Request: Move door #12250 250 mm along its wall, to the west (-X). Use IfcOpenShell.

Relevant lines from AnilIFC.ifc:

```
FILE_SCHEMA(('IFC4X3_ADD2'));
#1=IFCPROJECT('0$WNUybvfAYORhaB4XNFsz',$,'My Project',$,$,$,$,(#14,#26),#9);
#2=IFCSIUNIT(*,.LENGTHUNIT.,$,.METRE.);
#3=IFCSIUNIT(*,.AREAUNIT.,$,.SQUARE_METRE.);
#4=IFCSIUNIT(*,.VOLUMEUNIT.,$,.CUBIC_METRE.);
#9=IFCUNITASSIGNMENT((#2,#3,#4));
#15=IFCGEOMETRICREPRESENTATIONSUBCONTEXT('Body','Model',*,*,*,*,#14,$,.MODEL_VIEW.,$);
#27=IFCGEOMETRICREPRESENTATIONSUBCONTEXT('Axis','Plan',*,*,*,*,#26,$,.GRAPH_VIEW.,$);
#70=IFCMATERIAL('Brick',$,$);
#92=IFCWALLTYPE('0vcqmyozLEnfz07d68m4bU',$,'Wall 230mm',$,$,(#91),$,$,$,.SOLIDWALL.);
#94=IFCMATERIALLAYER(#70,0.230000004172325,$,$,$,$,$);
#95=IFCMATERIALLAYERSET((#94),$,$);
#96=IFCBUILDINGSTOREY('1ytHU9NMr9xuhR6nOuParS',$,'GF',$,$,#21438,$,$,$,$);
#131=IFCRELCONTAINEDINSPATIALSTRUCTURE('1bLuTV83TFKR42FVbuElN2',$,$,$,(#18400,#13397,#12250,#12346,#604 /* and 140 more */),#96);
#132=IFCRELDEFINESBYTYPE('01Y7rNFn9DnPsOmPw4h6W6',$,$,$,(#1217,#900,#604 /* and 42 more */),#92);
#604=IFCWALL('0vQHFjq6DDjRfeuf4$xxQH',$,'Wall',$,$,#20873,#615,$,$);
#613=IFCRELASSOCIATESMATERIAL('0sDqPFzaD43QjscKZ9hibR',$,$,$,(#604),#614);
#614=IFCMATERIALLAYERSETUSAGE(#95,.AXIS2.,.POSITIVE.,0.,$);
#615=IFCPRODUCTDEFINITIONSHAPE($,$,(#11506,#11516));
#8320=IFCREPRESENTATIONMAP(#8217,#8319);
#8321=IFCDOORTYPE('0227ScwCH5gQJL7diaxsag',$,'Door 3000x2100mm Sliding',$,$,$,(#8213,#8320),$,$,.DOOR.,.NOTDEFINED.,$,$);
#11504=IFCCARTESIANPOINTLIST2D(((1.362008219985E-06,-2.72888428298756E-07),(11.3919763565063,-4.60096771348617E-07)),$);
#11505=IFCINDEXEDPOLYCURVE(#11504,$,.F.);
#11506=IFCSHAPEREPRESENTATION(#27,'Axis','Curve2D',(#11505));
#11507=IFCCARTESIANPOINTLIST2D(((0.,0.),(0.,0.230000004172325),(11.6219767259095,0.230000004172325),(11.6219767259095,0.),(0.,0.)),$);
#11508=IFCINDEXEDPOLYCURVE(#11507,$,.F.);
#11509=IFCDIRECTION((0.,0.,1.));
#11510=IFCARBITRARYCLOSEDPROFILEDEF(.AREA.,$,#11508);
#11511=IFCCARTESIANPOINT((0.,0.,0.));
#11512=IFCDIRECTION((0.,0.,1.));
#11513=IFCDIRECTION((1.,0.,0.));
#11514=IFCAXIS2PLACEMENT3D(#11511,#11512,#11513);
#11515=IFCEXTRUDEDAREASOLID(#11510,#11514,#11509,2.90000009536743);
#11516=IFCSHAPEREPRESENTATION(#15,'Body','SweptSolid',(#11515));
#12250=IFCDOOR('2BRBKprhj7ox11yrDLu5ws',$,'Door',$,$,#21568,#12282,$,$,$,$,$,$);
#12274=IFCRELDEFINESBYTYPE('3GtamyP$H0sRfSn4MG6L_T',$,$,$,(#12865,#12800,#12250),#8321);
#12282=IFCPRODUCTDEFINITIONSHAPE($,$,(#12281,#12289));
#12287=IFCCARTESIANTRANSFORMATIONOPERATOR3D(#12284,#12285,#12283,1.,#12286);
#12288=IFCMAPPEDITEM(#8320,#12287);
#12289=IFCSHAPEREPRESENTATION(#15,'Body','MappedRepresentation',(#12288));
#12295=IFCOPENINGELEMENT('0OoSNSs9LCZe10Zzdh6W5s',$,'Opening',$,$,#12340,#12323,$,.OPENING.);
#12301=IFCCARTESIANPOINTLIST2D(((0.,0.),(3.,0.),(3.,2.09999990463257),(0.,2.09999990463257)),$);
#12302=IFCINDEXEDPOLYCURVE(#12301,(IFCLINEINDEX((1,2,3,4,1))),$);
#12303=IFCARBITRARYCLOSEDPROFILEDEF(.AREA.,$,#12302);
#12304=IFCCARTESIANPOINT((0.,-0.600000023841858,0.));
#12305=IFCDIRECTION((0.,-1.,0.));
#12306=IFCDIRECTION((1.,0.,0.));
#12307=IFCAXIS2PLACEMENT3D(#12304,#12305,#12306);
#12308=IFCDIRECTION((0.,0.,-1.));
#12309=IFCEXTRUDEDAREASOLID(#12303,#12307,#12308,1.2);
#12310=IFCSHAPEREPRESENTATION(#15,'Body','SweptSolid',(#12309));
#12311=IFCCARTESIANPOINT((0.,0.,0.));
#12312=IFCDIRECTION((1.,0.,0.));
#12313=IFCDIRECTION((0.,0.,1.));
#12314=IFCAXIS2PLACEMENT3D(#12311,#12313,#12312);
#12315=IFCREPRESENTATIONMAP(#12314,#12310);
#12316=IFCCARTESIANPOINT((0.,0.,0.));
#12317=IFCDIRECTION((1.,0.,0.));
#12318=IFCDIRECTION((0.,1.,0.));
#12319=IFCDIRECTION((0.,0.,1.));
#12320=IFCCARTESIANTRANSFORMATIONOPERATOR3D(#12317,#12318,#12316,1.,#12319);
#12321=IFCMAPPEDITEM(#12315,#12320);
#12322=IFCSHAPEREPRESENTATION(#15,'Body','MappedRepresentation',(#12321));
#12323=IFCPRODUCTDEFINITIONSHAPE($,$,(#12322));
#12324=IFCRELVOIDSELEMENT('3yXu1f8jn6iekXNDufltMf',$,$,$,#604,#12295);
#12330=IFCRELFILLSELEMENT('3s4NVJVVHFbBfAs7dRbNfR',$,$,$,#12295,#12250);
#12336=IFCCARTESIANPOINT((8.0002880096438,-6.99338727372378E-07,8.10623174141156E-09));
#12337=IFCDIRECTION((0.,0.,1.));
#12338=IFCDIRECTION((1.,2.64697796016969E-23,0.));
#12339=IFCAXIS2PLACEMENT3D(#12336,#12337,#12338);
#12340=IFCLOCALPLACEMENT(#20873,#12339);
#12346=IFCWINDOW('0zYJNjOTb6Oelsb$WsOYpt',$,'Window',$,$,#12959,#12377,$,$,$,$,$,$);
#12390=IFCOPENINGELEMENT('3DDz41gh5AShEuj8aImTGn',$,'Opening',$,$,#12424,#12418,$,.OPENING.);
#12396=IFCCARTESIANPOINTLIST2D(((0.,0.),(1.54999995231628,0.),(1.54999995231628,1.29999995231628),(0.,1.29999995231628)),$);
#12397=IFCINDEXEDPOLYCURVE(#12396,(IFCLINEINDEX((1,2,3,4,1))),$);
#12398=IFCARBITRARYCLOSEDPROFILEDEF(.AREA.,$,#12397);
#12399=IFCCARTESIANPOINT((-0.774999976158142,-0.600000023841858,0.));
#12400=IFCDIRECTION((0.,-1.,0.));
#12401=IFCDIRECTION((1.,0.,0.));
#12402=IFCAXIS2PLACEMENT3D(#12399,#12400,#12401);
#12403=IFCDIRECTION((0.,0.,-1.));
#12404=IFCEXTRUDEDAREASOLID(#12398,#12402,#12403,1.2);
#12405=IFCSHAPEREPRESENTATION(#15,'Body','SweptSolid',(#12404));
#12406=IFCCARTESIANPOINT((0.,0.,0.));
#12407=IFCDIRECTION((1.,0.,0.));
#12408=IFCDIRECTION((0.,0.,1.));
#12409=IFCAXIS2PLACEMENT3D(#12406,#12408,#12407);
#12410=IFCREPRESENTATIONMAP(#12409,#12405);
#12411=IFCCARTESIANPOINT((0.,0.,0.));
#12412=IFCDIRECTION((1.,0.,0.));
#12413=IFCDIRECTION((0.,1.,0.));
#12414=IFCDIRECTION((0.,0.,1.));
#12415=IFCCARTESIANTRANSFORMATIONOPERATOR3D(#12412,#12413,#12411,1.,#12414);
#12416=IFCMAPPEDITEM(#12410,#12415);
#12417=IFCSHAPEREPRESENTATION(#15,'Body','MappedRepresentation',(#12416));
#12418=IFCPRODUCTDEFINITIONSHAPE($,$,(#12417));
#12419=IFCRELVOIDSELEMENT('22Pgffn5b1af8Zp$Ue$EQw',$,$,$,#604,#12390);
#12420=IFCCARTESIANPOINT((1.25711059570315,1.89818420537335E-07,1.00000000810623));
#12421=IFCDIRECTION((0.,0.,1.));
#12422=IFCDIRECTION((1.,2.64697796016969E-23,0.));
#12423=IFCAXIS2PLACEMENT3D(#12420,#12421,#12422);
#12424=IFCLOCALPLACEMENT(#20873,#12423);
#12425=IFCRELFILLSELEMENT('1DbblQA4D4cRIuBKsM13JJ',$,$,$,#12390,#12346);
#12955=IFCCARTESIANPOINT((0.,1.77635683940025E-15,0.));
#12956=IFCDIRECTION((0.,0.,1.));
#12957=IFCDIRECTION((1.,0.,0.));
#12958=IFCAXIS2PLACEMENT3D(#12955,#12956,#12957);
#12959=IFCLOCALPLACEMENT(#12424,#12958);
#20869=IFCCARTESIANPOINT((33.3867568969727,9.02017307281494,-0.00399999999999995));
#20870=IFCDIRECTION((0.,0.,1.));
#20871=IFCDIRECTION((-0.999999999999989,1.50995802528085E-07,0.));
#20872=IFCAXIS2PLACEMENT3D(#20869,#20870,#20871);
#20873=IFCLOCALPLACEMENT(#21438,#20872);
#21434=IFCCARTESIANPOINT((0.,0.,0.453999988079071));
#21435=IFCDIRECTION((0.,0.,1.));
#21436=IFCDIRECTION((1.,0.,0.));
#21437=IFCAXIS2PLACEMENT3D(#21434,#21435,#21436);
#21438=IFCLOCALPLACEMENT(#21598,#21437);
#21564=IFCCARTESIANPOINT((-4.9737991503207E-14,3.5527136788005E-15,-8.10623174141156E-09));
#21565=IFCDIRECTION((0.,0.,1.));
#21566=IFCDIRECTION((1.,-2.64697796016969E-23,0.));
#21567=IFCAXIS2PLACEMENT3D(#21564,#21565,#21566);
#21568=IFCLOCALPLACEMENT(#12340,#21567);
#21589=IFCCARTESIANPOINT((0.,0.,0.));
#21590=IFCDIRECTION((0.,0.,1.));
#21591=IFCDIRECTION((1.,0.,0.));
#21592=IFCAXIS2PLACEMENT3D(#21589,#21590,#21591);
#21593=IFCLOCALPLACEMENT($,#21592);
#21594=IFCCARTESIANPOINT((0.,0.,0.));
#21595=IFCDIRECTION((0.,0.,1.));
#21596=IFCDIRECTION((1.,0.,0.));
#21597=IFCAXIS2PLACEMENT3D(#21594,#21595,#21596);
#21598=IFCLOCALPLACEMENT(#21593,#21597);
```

```python
import ifcopenshell
import ifcopenshell.api.geometry
import ifcopenshell.util.placement
import ifcopenshell.util.unit

model = ifcopenshell.open("AnilIFC.ifc")
unit_scale = ifcopenshell.util.unit.calculate_unit_scale(model)

door = model.by_guid("2BRBKprhj7ox11yrDLu5ws")
opening = door.FillsVoids[0].RelatingOpeningElement
wall = opening.VoidsElements[0].RelatingBuildingElement

wall_matrix = ifcopenshell.util.placement.get_local_placement(wall.ObjectPlacement)
shift = wall_matrix[:3, 0] * 0.25 / unit_scale
before = ifcopenshell.util.placement.get_local_placement(door.ObjectPlacement)[:3, 3].copy()

# The door is placed relative to its opening, so it follows when the opening moves.
matrix = ifcopenshell.util.placement.get_local_placement(opening.ObjectPlacement)
matrix[:3, 3] += shift
ifcopenshell.api.geometry.edit_object_placement(
    model, product=opening, matrix=matrix, is_si=False, should_transform_children=True
)

after = ifcopenshell.util.placement.get_local_placement(door.ObjectPlacement)[:3, 3]
print("door moved by", (after - before).round(3) + 0.0)

model.write("AnilIFC_updated.ifc")
```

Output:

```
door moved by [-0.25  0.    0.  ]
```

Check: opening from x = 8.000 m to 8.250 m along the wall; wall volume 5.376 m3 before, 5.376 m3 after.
